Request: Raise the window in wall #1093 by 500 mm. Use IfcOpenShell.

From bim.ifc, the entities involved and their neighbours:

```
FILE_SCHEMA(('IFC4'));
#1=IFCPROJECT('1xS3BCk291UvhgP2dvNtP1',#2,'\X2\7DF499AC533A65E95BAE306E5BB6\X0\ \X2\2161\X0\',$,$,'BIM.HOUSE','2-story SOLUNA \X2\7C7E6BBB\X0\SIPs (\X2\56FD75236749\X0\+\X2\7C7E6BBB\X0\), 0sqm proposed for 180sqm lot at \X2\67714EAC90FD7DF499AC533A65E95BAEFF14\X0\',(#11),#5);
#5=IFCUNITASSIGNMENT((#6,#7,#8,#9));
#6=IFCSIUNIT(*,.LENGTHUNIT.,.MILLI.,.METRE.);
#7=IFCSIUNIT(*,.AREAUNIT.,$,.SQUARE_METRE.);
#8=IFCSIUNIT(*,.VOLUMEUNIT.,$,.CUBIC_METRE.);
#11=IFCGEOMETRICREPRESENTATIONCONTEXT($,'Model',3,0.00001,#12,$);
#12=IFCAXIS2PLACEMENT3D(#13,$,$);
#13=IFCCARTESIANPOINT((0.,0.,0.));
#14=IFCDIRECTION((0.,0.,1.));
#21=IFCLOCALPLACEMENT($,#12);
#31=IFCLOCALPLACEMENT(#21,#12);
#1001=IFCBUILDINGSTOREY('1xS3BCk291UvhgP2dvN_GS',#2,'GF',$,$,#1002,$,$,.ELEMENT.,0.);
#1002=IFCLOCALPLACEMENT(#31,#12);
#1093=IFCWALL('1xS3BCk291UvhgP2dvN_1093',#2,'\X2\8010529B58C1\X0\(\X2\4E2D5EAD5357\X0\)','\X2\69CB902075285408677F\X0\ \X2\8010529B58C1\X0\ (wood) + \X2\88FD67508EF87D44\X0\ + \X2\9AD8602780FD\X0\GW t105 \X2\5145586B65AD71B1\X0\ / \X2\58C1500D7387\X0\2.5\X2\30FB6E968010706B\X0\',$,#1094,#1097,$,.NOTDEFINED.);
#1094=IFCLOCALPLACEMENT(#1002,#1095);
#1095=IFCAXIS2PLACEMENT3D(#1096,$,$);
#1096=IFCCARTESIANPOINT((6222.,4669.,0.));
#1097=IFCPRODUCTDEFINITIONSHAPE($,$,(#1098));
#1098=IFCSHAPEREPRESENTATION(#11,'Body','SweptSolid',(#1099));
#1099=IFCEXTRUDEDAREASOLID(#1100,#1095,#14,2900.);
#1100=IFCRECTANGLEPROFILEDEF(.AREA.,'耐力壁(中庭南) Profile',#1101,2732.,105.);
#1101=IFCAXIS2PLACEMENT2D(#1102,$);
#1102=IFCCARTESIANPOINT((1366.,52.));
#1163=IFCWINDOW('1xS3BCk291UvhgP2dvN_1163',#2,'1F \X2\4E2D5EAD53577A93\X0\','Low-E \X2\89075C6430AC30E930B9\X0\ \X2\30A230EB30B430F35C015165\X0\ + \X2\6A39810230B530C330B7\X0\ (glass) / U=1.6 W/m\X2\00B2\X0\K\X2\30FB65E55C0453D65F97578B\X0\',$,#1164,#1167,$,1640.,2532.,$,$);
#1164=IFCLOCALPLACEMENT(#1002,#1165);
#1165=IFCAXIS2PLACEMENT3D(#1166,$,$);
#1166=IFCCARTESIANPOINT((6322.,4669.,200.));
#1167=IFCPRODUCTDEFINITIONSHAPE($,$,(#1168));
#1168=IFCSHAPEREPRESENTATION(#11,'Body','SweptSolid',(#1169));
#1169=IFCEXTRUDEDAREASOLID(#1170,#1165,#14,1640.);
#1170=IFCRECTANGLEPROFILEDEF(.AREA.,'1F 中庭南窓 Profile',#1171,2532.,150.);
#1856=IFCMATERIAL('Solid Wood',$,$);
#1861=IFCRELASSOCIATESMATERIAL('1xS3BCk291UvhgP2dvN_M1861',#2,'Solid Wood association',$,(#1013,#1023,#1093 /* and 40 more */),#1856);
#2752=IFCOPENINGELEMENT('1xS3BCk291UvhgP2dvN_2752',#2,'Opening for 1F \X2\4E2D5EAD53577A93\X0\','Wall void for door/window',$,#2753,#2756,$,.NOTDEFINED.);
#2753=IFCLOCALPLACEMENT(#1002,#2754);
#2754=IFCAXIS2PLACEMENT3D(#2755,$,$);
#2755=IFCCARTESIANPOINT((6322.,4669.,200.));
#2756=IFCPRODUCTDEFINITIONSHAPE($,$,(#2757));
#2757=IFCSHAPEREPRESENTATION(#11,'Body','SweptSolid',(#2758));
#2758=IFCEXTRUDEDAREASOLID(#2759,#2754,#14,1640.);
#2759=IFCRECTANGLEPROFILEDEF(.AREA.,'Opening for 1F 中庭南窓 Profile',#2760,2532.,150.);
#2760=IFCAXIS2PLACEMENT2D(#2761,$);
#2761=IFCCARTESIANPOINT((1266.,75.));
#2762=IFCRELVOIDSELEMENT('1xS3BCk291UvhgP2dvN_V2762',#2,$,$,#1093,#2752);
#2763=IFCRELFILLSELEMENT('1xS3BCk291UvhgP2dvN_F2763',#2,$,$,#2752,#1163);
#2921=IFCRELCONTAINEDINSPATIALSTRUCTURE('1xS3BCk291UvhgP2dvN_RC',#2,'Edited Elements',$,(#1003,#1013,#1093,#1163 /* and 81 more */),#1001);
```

```python
import numpy as np
import ifcopenshell
import ifcopenshell.api.geometry
import ifcopenshell.util.placement
import ifcopenshell.util.unit

model = ifcopenshell.open("bim.ifc")
unit_scale = ifcopenshell.util.unit.calculate_unit_scale(model)

window = model.by_guid("1xS3BCk291UvhgP2dvN_1163")
opening = window.FillsVoids[0].RelatingOpeningElement
dz = 0.5 / unit_scale

shift = np.array([0.0, 0.0, dz])
# The window is not placed relative to its opening, so move both.
for product in (opening, window):
    matrix = ifcopenshell.util.placement.get_local_placement(product.ObjectPlacement)
    matrix[:3, 3] += shift
    ifcopenshell.api.geometry.edit_object_placement(model, product=product, matrix=matrix, is_si=False)

print(f"moved by {dz * unit_scale:+.3f} m")

model.write("bim_edited.ifc")
```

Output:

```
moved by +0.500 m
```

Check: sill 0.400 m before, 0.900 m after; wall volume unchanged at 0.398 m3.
